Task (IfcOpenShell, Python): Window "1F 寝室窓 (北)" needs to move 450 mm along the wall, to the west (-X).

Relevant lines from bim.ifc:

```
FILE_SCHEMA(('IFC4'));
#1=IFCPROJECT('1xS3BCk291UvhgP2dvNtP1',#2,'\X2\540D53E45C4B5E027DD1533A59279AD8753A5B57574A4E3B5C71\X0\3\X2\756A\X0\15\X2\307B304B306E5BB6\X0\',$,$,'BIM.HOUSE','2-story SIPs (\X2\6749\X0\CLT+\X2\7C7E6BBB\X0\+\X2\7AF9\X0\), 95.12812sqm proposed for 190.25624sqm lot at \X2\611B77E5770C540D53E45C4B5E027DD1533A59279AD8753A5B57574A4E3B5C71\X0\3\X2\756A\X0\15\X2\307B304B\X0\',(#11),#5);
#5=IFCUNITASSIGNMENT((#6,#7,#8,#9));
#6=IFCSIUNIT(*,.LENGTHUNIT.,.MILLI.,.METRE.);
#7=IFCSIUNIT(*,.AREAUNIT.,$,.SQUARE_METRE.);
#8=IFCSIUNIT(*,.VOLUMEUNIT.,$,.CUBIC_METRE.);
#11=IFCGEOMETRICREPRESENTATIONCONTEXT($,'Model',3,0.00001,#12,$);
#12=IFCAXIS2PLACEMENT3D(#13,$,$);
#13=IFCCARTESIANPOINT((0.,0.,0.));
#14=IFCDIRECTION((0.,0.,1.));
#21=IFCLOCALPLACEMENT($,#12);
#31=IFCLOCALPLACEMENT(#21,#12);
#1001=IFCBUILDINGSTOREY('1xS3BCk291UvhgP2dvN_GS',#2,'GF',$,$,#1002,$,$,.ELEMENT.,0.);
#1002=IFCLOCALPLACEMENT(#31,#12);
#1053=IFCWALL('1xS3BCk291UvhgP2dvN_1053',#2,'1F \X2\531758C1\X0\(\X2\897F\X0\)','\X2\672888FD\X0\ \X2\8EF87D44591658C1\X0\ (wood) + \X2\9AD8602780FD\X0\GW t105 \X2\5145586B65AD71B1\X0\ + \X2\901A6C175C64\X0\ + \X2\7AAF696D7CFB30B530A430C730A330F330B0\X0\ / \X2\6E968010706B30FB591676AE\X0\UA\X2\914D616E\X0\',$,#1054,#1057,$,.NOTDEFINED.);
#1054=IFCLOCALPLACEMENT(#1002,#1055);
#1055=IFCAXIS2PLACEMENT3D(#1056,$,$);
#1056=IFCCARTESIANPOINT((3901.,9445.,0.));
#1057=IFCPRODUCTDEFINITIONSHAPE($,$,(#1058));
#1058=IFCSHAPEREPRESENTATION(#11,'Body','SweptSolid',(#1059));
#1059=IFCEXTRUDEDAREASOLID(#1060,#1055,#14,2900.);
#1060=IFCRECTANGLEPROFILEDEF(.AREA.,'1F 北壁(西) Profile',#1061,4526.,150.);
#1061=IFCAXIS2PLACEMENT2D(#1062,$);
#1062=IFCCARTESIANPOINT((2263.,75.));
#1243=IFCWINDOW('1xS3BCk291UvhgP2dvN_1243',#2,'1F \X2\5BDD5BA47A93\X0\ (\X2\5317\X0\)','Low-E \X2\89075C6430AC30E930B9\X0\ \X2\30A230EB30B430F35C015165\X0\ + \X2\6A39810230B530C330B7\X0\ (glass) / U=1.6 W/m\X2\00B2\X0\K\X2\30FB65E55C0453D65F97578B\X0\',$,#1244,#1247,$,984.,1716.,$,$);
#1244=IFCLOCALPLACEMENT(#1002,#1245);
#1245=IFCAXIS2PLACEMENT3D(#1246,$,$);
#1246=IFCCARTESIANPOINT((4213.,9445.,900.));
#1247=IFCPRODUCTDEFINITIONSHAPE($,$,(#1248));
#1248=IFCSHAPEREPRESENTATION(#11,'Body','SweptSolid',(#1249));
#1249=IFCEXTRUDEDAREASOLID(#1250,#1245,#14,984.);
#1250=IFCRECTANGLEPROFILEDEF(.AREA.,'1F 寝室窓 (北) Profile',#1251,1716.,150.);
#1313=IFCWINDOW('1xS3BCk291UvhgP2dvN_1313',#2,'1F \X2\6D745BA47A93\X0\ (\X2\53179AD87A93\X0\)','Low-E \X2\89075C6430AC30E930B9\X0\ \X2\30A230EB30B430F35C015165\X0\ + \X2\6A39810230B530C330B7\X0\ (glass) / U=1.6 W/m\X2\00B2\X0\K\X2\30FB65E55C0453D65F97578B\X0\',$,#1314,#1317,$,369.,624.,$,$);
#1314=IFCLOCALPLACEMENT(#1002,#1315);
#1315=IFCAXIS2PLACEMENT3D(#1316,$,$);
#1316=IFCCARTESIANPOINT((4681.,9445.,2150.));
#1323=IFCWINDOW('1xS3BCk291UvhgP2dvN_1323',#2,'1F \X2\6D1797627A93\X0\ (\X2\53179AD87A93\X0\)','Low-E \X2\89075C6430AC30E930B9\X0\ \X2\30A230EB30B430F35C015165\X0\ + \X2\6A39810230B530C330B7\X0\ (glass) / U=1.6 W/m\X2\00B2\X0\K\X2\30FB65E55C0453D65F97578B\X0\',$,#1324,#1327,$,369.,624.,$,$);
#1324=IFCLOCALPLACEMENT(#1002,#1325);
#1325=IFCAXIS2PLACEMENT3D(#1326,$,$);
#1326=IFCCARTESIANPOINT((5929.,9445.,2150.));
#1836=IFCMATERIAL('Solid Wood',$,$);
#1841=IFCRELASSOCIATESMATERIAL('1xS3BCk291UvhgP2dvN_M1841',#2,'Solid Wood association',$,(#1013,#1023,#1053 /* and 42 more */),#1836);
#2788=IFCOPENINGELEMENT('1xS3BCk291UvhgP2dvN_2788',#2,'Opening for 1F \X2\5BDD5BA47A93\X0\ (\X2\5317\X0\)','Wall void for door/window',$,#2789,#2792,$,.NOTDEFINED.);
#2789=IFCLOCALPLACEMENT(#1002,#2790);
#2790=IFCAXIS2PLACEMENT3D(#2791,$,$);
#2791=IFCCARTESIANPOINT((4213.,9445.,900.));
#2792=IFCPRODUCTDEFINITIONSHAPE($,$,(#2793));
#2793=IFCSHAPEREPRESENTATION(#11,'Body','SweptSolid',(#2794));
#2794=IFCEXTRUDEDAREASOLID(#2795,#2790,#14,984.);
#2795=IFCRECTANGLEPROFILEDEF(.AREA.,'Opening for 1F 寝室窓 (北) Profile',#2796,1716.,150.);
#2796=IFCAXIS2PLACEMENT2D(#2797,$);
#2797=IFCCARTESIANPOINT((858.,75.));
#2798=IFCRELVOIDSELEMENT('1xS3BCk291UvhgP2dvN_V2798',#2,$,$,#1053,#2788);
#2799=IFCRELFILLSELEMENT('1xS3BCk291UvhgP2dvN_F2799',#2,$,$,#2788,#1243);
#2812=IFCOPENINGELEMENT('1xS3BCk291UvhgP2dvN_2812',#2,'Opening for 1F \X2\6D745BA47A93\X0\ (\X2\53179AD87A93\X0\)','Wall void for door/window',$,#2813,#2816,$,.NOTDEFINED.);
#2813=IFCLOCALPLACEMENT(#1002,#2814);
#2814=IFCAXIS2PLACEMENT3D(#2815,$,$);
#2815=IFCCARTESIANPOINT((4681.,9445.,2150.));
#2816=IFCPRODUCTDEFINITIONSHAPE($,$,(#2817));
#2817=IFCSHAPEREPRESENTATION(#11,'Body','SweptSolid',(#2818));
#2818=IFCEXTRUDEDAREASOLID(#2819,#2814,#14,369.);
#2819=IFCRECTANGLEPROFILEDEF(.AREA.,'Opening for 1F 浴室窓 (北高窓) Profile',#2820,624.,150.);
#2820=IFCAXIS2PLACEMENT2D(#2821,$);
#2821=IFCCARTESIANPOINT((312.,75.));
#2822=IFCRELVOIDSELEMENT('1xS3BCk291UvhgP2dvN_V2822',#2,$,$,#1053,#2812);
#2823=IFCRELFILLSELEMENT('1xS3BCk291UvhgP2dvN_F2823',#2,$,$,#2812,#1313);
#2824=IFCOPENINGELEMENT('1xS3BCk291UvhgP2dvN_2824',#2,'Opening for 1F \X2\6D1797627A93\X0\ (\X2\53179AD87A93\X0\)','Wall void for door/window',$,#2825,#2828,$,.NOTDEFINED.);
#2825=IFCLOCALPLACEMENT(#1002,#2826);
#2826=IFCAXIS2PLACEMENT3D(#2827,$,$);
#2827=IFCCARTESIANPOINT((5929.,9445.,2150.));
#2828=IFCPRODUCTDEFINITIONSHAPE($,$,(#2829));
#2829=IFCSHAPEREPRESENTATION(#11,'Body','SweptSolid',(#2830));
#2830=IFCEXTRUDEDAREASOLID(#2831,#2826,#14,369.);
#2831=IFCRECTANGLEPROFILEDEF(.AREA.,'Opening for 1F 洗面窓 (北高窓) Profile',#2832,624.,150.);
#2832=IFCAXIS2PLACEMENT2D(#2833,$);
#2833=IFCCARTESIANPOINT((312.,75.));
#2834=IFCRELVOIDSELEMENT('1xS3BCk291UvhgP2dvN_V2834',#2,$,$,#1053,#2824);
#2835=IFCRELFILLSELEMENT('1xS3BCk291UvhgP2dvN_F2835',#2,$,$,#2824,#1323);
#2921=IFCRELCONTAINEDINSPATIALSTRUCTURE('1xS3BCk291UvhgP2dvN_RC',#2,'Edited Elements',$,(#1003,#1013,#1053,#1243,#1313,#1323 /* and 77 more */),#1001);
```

```python
import ifcopenshell
import ifcopenshell.api.geometry
import ifcopenshell.util.placement
import ifcopenshell.util.unit

model = ifcopenshell.open("bim.ifc")
unit_scale = ifcopenshell.util.unit.calculate_unit_scale(model)

window = model.by_guid("1xS3BCk291UvhgP2dvN_1243")
opening = window.FillsVoids[0].RelatingOpeningElement
wall = opening.VoidsElements[0].RelatingBuildingElement

wall_matrix = ifcopenshell.util.placement.get_local_placement(wall.ObjectPlacement)
shift = wall_matrix[:3, 0] * -0.45 / unit_scale
before = ifcopenshell.util.placement.get_local_placement(window.ObjectPlacement)[:3, 3].copy()

# The window is not placed relative to its opening, so move both.
for product in (opening, window):
    matrix = ifcopenshell.util.placement.get_local_placement(product.ObjectPlacement)
    matrix[:3, 3] += shift
    ifcopenshell.api.geometry.edit_object_placement(model, product=product, matrix=matrix, is_si=False)

after = ifcopenshell.util.placement.get_local_placement(window.ObjectPlacement)[:3, 3]
print("window moved by", (after - before).round(3) + 0.0)

model.write("bim_rev.ifc")
```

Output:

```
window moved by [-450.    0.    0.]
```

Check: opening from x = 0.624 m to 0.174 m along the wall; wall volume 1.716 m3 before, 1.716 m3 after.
